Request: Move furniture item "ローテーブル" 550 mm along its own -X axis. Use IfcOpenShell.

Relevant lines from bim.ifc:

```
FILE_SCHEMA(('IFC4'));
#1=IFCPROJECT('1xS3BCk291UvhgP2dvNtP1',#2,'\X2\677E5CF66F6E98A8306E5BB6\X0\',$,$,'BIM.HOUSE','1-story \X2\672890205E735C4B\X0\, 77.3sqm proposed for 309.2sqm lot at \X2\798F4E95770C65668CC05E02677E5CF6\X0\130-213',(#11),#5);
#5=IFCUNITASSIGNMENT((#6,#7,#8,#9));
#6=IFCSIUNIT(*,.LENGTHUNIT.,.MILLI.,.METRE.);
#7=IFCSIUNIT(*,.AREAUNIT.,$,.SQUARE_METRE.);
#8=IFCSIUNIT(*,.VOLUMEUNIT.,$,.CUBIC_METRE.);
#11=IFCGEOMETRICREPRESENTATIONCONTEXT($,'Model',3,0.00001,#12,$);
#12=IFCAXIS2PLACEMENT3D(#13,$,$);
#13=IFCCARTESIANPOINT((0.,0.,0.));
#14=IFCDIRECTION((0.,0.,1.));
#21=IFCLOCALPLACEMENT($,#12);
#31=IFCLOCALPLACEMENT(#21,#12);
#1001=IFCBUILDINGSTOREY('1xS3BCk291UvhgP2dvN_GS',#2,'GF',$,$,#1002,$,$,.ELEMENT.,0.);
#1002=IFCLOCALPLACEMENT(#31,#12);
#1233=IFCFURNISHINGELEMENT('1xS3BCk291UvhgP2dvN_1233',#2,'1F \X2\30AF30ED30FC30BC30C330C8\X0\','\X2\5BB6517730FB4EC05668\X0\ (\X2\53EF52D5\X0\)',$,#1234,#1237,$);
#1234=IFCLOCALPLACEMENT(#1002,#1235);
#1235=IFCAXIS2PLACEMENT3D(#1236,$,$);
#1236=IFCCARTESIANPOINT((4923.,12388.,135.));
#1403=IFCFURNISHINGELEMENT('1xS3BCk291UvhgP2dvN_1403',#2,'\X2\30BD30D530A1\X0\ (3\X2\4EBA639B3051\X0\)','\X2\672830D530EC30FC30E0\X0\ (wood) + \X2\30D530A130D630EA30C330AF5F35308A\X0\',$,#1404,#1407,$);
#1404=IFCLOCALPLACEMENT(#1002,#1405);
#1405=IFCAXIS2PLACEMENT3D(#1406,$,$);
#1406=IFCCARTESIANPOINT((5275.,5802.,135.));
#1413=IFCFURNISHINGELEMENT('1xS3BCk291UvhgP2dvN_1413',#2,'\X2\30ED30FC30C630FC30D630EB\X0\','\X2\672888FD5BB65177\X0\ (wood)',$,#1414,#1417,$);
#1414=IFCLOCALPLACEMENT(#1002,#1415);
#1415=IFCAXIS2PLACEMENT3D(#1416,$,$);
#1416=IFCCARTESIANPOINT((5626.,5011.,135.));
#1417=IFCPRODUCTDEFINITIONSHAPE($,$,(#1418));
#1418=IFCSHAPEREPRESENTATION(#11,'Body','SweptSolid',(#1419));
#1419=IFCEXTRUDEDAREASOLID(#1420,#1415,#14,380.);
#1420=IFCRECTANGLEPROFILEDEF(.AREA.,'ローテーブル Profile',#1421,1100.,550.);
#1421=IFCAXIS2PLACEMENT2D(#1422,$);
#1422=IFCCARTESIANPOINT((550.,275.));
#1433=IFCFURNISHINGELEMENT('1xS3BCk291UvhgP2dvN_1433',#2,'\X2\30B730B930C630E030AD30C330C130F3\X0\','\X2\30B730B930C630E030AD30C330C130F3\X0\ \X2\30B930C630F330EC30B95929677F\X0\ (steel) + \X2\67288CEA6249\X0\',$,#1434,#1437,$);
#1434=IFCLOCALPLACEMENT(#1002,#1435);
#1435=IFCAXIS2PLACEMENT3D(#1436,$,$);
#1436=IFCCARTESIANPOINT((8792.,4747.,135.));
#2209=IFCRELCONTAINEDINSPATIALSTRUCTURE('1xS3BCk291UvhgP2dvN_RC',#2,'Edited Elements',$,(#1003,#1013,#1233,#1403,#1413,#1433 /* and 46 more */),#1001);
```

```python
import ifcopenshell
import ifcopenshell.api.geometry
import ifcopenshell.util.placement
import ifcopenshell.util.unit

model = ifcopenshell.open("bim.ifc")
unit_scale = ifcopenshell.util.unit.calculate_unit_scale(model)

item = model.by_guid("1xS3BCk291UvhgP2dvN_1413")
matrix = ifcopenshell.util.placement.get_local_placement(item.ObjectPlacement)
matrix[:3, 3] -= matrix[:3, 0] * 0.55 / unit_scale
ifcopenshell.api.geometry.edit_object_placement(model, product=item, matrix=matrix, is_si=False)

print(ifcopenshell.util.placement.get_local_placement(item.ObjectPlacement).round(3) + 0.0)

model.write("bim-out.ifc")
```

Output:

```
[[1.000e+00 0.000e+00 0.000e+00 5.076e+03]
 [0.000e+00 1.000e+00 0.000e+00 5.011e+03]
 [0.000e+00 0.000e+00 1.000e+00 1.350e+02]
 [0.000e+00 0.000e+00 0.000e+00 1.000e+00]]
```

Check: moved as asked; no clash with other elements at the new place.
